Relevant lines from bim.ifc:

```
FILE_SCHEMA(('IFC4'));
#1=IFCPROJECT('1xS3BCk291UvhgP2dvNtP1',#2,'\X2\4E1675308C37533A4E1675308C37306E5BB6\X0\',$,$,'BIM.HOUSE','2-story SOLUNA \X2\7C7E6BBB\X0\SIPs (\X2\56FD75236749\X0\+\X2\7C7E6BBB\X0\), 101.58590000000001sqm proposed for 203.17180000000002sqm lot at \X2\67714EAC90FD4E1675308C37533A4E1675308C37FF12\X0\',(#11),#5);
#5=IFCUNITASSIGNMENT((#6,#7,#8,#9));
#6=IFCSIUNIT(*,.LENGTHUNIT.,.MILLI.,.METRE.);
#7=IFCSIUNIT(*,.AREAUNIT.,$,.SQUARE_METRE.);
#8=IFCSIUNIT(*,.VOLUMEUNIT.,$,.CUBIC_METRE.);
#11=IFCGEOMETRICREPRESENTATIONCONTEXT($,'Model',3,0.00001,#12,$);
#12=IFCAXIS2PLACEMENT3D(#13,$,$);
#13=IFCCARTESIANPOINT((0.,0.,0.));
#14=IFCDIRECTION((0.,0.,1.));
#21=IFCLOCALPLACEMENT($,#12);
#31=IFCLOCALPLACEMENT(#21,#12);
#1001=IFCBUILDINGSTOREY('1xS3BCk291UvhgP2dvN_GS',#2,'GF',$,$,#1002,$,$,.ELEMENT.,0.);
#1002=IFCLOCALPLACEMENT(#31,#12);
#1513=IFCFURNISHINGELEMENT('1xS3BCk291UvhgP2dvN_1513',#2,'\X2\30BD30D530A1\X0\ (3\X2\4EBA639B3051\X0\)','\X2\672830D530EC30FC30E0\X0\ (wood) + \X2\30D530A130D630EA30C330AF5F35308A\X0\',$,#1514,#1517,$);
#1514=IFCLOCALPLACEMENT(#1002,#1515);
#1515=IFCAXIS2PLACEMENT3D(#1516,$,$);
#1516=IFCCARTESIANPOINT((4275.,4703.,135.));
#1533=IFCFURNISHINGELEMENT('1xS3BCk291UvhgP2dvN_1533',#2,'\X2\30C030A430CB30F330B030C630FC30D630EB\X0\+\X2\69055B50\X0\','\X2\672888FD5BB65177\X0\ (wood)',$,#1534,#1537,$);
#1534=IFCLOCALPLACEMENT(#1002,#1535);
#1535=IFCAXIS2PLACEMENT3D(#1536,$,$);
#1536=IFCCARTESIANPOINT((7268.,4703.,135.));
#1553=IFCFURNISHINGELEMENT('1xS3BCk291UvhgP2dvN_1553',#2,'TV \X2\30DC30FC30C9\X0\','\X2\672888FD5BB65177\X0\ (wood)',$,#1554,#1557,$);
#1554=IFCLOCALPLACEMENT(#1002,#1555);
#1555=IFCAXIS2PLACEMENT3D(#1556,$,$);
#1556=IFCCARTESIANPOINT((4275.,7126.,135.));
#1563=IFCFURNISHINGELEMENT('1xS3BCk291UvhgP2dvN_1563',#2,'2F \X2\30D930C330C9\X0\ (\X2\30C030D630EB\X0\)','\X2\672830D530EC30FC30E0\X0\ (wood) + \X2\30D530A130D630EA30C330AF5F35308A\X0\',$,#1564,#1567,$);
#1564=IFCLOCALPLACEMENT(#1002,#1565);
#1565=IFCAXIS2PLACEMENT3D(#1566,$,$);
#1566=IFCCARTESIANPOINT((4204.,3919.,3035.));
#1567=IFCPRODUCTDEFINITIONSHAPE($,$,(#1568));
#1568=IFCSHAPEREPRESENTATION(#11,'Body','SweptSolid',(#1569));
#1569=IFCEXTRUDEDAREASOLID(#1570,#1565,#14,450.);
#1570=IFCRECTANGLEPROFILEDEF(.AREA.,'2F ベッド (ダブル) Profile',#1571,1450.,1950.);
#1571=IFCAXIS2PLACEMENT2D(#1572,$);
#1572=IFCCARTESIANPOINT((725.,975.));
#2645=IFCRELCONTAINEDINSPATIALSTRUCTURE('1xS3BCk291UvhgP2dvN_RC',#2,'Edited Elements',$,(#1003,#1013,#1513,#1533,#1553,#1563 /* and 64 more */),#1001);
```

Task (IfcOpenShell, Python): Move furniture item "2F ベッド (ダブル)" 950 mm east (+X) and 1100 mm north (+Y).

```python
import ifcopenshell
import ifcopenshell.api.geometry
import ifcopenshell.util.placement

model = ifcopenshell.open("bim.ifc")

item = model.by_guid("1xS3BCk291UvhgP2dvN_1563")
matrix = ifcopenshell.util.placement.get_local_placement(item.ObjectPlacement)
matrix[0, 3] += 950.0
matrix[1, 3] += 1100.0
ifcopenshell.api.geometry.edit_object_placement(model, product=item, matrix=matrix, is_si=False)

print(ifcopenshell.util.placement.get_local_placement(item.ObjectPlacement).round(3) + 0.0)

model.write("bim_v2.ifc")
```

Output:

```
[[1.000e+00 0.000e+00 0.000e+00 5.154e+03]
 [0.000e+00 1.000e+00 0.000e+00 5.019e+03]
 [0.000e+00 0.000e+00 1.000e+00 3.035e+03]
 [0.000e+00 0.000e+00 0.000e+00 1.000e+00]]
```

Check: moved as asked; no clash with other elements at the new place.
